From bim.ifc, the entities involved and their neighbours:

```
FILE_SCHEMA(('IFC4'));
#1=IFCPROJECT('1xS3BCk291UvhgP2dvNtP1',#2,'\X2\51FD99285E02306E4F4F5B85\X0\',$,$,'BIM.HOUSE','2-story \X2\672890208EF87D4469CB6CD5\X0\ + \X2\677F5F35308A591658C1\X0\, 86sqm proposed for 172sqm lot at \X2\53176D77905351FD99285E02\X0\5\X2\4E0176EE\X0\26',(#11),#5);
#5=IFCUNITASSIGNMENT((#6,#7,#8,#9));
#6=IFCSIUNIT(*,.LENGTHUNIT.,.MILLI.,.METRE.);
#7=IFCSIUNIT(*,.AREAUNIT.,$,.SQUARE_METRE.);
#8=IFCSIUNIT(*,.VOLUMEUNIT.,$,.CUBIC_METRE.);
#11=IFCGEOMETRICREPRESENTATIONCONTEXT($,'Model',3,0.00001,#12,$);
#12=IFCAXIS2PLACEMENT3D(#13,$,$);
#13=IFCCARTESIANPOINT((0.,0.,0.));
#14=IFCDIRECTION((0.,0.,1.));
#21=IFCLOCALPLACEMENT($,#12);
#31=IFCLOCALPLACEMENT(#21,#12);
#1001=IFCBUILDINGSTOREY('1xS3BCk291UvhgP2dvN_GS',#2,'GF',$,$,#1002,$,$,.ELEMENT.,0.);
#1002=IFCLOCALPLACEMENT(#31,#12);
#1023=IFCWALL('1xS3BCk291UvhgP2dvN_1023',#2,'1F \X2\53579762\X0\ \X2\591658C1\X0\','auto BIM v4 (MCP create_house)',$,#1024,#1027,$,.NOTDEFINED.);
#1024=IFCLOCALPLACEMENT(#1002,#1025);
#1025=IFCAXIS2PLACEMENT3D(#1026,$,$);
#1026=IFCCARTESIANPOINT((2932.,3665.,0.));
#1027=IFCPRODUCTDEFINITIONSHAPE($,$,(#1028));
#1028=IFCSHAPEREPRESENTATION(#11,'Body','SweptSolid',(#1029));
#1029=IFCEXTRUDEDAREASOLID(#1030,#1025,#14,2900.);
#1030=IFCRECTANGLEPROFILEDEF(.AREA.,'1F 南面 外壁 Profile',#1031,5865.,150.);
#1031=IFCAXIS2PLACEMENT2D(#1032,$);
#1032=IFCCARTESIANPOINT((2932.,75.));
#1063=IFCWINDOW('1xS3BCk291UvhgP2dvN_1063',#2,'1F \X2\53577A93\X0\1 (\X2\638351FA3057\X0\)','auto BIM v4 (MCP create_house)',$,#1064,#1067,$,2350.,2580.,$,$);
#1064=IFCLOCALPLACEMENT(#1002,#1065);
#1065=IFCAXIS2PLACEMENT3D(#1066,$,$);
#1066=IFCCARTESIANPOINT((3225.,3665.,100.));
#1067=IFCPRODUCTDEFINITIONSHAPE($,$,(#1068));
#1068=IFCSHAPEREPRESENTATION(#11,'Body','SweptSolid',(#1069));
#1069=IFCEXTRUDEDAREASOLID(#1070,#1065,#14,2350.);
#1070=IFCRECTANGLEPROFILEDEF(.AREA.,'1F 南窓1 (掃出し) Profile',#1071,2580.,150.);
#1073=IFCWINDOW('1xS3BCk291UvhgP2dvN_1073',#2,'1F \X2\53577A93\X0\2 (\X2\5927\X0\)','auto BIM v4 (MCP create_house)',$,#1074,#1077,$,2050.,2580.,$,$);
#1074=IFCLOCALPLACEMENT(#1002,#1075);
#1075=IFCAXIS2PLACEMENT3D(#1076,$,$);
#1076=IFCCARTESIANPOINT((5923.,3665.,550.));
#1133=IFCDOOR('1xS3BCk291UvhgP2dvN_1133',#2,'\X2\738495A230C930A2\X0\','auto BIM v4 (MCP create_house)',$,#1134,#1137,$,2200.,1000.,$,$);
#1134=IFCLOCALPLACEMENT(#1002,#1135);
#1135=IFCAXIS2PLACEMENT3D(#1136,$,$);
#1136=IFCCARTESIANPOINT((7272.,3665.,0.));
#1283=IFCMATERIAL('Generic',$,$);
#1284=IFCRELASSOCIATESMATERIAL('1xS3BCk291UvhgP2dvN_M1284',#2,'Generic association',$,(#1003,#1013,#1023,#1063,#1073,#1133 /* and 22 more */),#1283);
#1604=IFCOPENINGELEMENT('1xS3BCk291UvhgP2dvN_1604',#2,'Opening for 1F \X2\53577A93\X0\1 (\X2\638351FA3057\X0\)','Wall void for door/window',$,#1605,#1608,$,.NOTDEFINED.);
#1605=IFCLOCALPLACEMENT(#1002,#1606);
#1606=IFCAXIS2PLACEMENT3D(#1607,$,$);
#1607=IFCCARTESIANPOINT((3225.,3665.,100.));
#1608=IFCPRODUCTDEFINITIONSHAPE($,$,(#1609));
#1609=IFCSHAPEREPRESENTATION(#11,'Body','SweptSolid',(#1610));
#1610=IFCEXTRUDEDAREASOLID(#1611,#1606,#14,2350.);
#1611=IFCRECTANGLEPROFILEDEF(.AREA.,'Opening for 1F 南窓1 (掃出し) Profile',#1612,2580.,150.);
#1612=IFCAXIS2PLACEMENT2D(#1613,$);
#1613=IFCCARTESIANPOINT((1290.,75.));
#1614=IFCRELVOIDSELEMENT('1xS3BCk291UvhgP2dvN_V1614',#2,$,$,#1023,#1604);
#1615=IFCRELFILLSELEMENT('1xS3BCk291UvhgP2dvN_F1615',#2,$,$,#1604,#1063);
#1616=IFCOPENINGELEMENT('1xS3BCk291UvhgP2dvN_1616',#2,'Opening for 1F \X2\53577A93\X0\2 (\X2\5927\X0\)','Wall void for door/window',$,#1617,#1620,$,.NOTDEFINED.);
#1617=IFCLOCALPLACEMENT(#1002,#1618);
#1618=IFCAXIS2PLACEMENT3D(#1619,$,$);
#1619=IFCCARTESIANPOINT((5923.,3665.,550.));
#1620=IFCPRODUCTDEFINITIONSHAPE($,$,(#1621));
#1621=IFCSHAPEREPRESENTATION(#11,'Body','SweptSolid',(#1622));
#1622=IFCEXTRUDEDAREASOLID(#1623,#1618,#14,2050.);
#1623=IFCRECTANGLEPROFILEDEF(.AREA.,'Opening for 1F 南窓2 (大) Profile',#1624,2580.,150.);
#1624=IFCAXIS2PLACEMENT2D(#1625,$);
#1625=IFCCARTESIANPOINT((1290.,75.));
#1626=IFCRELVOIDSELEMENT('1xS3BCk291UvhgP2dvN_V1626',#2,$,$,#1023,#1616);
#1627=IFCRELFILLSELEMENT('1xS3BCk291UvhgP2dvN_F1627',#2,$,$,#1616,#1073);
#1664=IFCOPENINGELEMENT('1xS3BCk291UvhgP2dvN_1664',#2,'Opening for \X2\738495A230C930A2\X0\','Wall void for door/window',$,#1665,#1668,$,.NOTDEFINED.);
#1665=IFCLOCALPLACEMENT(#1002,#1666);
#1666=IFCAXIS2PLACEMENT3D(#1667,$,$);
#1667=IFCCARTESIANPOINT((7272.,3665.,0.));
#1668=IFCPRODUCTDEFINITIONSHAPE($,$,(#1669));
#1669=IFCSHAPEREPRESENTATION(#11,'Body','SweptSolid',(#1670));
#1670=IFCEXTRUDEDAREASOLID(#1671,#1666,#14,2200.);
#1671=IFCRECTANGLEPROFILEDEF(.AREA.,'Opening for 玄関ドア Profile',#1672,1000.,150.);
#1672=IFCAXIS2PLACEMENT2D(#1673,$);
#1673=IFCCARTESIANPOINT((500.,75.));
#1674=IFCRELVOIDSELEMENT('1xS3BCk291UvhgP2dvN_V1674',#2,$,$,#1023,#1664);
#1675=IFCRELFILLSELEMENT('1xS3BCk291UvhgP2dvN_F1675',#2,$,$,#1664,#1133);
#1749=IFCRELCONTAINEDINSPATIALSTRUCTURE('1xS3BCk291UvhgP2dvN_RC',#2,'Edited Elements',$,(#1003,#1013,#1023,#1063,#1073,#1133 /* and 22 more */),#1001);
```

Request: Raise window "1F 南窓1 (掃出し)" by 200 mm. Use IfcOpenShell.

```python
import numpy as np
import ifcopenshell
import ifcopenshell.api.geometry
import ifcopenshell.util.placement
import ifcopenshell.util.unit

model = ifcopenshell.open("bim.ifc")
unit_scale = ifcopenshell.util.unit.calculate_unit_scale(model)

window = model.by_guid("1xS3BCk291UvhgP2dvN_1063")
opening = window.FillsVoids[0].RelatingOpeningElement
dz = 0.2 / unit_scale

shift = np.array([0.0, 0.0, dz])
# The window is not placed relative to its opening, so move both.
for product in (opening, window):
    matrix = ifcopenshell.util.placement.get_local_placement(product.ObjectPlacement)
    matrix[:3, 3] += shift
    ifcopenshell.api.geometry.edit_object_placement(model, product=product, matrix=matrix, is_si=False)

print(f"moved by {dz * unit_scale:+.3f} m")

model.write("bim_edited.ifc")
```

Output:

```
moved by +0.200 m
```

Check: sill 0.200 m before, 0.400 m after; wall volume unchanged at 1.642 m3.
